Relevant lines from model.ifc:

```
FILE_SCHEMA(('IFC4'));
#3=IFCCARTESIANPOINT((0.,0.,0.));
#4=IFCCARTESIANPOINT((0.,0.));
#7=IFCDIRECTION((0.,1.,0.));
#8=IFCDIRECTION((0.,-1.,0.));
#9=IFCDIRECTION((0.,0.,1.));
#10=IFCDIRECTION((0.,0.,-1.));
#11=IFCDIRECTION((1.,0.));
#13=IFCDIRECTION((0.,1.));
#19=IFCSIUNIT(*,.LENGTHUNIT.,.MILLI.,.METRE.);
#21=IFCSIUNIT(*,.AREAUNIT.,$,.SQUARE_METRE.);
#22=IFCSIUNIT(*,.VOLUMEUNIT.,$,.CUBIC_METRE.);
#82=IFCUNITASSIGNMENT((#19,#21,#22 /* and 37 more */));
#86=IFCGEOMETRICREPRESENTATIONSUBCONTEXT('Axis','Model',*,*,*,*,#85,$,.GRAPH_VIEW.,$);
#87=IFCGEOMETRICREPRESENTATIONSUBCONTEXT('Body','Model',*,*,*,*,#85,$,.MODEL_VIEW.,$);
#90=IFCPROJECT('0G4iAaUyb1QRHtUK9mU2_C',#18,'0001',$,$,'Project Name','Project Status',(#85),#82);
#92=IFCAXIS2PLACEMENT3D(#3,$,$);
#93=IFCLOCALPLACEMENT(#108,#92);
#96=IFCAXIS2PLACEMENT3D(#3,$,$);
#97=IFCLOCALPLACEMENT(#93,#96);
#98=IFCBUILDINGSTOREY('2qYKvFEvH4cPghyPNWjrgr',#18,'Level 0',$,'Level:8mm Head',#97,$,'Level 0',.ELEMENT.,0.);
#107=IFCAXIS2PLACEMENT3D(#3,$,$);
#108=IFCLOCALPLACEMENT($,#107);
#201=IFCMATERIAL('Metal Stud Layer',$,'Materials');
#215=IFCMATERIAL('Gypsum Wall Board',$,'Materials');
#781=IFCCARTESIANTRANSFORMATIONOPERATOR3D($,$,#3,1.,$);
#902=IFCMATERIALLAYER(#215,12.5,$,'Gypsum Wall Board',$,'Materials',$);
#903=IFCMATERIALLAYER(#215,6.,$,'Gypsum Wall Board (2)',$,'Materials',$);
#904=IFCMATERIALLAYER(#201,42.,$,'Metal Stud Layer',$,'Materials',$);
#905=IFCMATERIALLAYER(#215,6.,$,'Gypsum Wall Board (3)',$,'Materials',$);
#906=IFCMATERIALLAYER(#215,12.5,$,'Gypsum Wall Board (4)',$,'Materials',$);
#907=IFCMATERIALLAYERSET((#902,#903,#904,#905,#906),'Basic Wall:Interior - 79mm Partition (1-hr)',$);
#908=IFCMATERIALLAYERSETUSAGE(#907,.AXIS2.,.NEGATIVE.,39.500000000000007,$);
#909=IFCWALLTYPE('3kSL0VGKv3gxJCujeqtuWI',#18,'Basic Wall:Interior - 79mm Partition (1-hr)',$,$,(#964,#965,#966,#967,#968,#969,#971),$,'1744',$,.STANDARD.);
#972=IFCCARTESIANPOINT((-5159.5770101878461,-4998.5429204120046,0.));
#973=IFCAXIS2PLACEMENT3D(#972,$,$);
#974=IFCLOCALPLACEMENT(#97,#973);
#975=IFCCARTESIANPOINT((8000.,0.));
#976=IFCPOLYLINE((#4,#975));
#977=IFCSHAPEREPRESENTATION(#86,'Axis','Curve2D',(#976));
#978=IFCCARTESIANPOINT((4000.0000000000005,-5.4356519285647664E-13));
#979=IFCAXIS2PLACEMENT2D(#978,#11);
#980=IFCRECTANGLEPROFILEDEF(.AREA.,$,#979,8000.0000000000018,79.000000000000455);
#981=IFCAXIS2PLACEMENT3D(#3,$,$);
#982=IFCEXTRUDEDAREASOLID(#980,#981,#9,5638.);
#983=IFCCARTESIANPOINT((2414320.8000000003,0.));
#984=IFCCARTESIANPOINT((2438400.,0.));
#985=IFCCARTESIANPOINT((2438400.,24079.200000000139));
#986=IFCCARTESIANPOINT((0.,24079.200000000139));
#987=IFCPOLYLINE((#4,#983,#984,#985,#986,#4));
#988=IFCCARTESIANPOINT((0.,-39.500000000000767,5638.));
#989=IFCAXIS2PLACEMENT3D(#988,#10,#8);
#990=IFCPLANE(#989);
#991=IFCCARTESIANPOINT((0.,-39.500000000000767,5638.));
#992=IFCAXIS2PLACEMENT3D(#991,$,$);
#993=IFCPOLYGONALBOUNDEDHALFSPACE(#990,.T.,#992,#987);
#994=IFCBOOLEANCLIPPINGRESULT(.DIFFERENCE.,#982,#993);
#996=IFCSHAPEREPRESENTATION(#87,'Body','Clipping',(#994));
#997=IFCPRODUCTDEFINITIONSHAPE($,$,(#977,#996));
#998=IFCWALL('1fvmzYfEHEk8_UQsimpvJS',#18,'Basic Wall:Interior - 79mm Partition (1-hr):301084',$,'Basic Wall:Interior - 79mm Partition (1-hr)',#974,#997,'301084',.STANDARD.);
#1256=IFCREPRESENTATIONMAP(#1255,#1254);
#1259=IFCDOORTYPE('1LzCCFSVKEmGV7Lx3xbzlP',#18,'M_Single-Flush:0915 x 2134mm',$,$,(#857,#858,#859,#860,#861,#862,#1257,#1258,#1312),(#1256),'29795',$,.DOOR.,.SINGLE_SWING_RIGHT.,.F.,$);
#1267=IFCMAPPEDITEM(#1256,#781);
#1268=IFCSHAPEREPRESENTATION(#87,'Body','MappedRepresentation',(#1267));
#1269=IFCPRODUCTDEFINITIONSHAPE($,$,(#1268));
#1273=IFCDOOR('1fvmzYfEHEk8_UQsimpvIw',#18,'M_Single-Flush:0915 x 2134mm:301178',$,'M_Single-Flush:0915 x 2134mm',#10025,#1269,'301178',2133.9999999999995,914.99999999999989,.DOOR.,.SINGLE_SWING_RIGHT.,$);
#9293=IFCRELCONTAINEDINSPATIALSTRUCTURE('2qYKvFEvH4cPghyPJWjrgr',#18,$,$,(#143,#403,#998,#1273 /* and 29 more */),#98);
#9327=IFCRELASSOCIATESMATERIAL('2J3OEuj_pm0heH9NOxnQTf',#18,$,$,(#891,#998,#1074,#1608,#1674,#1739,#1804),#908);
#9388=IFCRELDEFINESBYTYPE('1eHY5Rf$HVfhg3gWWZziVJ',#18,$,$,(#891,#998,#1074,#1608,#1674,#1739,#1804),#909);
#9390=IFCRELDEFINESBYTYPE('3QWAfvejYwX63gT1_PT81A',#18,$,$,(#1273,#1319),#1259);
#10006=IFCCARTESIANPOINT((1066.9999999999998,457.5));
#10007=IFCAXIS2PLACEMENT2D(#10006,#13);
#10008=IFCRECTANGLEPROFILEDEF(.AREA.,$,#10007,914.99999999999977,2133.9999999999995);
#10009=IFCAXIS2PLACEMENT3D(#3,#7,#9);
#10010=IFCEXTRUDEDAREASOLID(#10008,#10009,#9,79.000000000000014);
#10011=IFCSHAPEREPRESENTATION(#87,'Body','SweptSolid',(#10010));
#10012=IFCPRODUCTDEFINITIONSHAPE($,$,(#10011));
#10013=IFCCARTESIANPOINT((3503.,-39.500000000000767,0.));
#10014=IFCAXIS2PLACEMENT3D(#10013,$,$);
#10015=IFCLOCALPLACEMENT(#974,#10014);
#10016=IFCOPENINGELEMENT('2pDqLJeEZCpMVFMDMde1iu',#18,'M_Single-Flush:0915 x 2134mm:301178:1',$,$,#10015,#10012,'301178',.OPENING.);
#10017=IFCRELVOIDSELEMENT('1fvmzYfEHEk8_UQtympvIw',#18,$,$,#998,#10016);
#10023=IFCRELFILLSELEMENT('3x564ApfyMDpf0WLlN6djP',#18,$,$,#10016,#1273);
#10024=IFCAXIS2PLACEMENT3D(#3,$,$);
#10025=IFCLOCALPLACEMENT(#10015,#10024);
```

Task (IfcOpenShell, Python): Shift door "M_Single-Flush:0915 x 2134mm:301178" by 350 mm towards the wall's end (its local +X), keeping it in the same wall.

```python
import ifcopenshell
import ifcopenshell.api.geometry
import ifcopenshell.util.placement

model = ifcopenshell.open("model.ifc")

door = model.by_guid("1fvmzYfEHEk8_UQsimpvIw")
opening = door.FillsVoids[0].RelatingOpeningElement
wall = opening.VoidsElements[0].RelatingBuildingElement

wall_matrix = ifcopenshell.util.placement.get_local_placement(wall.ObjectPlacement)
shift = wall_matrix[:3, 0] * 350.0
before = ifcopenshell.util.placement.get_local_placement(door.ObjectPlacement)[:3, 3].copy()

# The door is placed relative to its opening, so it follows when the opening moves.
matrix = ifcopenshell.util.placement.get_local_placement(opening.ObjectPlacement)
matrix[:3, 3] += shift
ifcopenshell.api.geometry.edit_object_placement(
    model, product=opening, matrix=matrix, is_si=False, should_transform_children=True
)

after = ifcopenshell.util.placement.get_local_placement(door.ObjectPlacement)[:3, 3]
print("door moved by", (after - before).round(3) + 0.0)

model.write("model_edited.ifc")
```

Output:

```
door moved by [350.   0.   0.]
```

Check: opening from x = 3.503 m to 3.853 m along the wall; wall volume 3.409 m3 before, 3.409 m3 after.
